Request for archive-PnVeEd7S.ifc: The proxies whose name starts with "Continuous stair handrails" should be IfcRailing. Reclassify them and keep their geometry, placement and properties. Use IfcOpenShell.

First a look at what the model holds.

```python
import re

import ifcopenshell

model = ifcopenshell.open("archive-PnVeEd7S.ifc")
print(model.schema)
seen = {}
for e in model.by_type("IfcBuildingElementProxy"):
    name = re.sub(r":\d+(:\d+)?$", "", e.Name or "")  # drop the element id that some exporters append
    seen[name] = seen.get(name, 0) + 1
for name, count in sorted(seen.items()):
    print(count, "x", name)
```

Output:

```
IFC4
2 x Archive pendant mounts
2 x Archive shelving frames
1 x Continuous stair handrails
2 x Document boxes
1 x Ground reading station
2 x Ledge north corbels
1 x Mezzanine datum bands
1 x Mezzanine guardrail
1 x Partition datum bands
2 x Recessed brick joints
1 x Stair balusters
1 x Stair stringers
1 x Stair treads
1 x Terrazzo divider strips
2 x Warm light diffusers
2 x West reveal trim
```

```python
import ifcopenshell
import ifcopenshell.api.root

model = ifcopenshell.open("archive-PnVeEd7S.ifc")

proxies = [e.id() for e in model.by_type("IfcBuildingElementProxy") if (e.Name or "").startswith("Continuous stair handrails")]
for step_id in proxies:
    proxy = model.by_id(step_id)
    ifcopenshell.api.root.reassign_class(model, product=proxy, ifc_class="IfcRailing")

print(sum(model.by_id(i).is_a("IfcRailing") for i in proxies), "reclassified")

model.write("archive-PnVeEd7S_rev.ifc")
```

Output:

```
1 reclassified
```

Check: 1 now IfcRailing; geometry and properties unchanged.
